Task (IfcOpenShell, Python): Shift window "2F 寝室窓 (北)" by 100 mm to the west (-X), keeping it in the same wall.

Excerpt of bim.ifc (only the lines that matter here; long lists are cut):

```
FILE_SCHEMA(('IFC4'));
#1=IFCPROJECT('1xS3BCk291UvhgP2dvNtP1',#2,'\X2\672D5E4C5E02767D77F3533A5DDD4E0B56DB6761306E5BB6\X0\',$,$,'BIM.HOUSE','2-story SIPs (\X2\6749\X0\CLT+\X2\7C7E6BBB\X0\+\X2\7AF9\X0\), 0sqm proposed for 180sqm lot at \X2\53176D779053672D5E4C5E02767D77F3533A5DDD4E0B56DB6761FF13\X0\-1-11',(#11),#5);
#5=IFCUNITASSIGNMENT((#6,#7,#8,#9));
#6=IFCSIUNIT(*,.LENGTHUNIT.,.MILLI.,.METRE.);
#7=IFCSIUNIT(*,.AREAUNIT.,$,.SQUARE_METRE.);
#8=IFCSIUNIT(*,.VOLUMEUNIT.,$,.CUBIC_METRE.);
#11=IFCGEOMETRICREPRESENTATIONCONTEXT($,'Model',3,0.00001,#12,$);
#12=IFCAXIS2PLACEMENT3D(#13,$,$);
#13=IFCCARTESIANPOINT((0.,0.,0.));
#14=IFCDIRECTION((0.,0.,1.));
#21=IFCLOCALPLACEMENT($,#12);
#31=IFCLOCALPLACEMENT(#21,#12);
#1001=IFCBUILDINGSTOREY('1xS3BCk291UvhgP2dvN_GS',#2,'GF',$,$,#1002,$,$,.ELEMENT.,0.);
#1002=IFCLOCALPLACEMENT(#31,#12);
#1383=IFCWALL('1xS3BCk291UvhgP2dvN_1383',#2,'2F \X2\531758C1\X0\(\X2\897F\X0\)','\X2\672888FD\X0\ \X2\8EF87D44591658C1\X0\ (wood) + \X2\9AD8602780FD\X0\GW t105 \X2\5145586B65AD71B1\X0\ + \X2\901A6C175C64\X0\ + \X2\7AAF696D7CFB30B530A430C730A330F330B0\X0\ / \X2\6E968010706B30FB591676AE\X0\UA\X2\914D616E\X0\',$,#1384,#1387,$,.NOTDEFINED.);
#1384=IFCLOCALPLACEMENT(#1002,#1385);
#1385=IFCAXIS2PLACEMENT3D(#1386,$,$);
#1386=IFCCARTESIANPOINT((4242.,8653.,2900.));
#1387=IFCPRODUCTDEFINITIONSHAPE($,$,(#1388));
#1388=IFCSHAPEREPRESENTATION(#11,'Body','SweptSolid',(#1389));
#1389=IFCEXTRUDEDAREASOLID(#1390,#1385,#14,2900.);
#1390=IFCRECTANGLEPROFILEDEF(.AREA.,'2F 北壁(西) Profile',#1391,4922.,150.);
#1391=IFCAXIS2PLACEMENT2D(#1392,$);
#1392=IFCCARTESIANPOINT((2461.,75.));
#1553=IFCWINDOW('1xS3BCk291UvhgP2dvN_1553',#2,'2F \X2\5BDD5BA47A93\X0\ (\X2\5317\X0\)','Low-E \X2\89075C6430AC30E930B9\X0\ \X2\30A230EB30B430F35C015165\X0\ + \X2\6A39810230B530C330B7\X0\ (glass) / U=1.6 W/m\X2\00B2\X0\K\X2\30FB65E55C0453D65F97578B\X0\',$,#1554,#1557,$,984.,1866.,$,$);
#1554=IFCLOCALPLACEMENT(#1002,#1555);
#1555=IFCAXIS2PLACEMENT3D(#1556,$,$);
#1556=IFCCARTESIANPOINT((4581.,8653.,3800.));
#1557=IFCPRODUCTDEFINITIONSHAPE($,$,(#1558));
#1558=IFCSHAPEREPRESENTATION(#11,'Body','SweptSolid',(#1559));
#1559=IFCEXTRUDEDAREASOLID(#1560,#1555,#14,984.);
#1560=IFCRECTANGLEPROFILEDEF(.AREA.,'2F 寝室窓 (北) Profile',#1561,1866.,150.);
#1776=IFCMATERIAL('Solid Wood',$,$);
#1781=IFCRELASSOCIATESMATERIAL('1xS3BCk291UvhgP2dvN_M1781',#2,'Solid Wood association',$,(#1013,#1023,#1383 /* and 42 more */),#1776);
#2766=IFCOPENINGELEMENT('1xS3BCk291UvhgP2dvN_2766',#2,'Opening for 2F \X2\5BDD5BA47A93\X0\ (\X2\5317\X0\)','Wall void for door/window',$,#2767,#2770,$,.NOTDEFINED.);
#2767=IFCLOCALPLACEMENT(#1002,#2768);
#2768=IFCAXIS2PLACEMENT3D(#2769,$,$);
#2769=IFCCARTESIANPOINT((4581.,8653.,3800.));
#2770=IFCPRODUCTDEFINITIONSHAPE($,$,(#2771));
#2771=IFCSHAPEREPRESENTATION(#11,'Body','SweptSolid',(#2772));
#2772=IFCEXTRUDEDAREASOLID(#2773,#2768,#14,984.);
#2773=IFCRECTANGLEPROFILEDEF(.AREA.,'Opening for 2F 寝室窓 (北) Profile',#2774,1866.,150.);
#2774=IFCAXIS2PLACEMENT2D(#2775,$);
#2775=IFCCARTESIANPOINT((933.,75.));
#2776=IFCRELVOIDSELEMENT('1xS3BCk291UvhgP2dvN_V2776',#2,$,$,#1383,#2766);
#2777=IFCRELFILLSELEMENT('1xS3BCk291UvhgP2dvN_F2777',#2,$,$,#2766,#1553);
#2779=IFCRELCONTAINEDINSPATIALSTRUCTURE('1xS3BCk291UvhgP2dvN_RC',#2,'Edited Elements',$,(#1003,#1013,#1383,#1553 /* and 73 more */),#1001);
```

```python
import ifcopenshell
import ifcopenshell.api.geometry
import ifcopenshell.util.placement
import ifcopenshell.util.unit

model = ifcopenshell.open("bim.ifc")
unit_scale = ifcopenshell.util.unit.calculate_unit_scale(model)

window = model.by_guid("1xS3BCk291UvhgP2dvN_1553")
opening = window.FillsVoids[0].RelatingOpeningElement
wall = opening.VoidsElements[0].RelatingBuildingElement

wall_matrix = ifcopenshell.util.placement.get_local_placement(wall.ObjectPlacement)
shift = wall_matrix[:3, 0] * -0.1 / unit_scale
before = ifcopenshell.util.placement.get_local_placement(window.ObjectPlacement)[:3, 3].copy()

# The window is not placed relative to its opening, so move both.
for product in (opening, window):
    matrix = ifcopenshell.util.placement.get_local_placement(product.ObjectPlacement)
    matrix[:3, 3] += shift
    ifcopenshell.api.geometry.edit_object_placement(model, product=product, matrix=matrix, is_si=False)

after = ifcopenshell.util.placement.get_local_placement(window.ObjectPlacement)[:3, 3]
print("window moved by", (after - before).round(3) + 0.0)

model.write("bim-out.ifc")
```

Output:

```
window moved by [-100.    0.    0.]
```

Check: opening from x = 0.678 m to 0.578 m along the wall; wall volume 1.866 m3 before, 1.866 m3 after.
